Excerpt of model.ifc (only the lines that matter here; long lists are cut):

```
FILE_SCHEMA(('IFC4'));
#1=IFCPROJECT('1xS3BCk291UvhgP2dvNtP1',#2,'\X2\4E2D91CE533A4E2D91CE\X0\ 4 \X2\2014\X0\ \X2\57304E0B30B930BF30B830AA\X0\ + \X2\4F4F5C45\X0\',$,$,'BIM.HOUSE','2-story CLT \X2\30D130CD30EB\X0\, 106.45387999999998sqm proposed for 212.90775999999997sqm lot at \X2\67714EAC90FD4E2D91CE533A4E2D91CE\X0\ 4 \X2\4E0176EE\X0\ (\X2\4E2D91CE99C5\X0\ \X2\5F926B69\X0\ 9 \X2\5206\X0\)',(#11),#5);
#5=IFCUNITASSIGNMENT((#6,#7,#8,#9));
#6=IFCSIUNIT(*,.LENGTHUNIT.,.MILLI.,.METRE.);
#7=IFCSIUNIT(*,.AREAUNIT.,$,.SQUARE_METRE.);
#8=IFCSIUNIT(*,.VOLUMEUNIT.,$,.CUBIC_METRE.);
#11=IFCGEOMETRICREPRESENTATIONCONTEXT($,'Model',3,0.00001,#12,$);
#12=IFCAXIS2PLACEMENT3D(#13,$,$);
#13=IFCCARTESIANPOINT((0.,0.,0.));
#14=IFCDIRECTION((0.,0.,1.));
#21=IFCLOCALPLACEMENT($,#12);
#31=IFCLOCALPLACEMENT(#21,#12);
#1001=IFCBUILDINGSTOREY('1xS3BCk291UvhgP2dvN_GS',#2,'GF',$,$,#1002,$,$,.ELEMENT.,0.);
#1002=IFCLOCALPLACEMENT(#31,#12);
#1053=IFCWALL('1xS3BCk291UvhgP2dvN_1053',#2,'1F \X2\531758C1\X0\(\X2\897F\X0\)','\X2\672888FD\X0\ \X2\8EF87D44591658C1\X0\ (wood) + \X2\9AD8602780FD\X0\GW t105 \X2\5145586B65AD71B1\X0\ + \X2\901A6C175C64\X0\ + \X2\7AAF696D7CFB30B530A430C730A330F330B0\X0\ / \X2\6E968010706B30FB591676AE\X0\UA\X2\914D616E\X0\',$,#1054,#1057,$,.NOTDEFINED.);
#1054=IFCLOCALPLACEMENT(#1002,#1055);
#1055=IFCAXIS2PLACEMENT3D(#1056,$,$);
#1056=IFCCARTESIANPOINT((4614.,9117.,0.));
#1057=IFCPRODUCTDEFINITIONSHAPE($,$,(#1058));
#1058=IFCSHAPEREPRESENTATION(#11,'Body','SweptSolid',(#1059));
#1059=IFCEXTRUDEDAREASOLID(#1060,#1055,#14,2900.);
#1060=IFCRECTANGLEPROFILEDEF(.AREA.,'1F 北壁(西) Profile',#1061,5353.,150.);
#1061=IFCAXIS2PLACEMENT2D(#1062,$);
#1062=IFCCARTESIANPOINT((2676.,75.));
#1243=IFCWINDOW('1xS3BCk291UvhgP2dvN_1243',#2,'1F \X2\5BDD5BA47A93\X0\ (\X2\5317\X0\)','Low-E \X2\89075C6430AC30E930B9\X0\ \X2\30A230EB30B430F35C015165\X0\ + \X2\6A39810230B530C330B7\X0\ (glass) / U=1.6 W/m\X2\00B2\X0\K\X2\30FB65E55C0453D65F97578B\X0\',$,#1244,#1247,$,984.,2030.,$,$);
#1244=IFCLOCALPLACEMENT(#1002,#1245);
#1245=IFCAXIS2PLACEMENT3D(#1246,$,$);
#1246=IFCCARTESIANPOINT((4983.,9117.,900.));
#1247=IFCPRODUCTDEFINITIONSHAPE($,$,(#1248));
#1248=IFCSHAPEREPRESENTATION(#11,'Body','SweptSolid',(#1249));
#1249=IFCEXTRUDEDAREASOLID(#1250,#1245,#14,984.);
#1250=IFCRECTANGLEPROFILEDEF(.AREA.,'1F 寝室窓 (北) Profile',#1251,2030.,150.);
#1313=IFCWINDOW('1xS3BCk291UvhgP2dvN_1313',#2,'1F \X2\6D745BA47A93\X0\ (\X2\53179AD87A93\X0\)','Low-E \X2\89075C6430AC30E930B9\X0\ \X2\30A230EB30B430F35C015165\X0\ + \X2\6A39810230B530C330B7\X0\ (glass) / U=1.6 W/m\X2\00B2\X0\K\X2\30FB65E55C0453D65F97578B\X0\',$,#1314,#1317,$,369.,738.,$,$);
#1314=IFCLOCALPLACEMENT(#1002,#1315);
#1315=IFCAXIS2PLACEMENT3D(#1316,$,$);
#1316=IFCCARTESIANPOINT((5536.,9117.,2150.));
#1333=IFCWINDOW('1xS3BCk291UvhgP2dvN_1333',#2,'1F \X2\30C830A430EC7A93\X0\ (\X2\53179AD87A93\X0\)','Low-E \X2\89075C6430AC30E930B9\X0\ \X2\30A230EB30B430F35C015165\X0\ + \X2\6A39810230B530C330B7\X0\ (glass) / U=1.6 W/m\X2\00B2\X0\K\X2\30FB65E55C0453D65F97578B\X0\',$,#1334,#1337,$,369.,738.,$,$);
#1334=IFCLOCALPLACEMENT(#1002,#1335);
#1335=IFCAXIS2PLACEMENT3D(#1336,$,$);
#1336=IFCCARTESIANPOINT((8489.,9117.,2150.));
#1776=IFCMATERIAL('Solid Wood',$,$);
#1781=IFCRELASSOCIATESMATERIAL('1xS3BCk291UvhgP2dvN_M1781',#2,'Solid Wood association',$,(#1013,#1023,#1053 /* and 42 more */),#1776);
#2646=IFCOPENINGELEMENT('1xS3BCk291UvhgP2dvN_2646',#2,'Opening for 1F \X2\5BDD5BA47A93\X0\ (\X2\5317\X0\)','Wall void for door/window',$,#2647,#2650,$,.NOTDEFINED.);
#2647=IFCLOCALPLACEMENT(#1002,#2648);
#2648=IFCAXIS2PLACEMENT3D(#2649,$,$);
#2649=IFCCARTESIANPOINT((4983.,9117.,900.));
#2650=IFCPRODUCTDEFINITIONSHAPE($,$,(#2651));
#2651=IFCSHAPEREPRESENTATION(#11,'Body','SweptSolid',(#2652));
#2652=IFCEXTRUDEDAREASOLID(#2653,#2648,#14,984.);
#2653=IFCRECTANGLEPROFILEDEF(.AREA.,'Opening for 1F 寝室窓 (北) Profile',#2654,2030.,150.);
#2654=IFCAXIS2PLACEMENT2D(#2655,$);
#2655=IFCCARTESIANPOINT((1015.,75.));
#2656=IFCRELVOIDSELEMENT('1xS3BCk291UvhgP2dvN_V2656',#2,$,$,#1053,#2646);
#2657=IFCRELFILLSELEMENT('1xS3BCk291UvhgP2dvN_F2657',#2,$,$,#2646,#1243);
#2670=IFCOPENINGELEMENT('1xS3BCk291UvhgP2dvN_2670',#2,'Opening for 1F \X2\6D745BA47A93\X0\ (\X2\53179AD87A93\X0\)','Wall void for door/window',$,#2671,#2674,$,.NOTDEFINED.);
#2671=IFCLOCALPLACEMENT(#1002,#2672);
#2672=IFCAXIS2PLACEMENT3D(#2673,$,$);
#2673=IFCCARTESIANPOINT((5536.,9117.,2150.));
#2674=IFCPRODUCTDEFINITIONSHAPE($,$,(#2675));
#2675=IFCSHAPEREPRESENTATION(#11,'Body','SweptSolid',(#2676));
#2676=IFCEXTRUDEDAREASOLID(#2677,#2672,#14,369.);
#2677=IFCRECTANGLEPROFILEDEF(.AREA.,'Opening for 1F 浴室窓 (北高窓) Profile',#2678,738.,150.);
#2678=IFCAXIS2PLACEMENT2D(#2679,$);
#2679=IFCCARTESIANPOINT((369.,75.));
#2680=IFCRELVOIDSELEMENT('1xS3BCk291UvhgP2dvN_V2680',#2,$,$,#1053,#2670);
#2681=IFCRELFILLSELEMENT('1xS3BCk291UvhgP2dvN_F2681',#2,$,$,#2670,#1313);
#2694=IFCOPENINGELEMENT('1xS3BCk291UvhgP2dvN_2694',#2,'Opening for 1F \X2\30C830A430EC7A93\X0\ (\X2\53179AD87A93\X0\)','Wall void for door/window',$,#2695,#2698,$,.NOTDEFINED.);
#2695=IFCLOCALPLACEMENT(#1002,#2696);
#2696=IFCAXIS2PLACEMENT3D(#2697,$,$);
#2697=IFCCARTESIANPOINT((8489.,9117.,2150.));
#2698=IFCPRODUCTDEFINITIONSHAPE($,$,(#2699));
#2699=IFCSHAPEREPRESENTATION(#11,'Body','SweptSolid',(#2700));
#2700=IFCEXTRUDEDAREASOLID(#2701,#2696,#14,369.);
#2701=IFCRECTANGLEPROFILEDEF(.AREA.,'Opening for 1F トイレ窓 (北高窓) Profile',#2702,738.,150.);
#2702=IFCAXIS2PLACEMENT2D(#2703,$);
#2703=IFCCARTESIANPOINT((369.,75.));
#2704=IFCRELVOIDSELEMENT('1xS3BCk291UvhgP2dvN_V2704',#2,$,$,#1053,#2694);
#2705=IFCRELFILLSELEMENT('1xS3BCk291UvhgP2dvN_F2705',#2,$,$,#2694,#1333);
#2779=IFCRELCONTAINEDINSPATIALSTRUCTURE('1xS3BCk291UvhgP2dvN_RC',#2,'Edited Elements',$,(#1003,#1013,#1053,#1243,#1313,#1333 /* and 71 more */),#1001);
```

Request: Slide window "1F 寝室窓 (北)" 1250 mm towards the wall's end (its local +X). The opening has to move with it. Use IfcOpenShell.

```python
import ifcopenshell
import ifcopenshell.api.geometry
import ifcopenshell.util.placement
import ifcopenshell.util.unit

model = ifcopenshell.open("model.ifc")
unit_scale = ifcopenshell.util.unit.calculate_unit_scale(model)

window = model.by_id(1243)
opening = window.FillsVoids[0].RelatingOpeningElement
wall = opening.VoidsElements[0].RelatingBuildingElement

wall_matrix = ifcopenshell.util.placement.get_local_placement(wall.ObjectPlacement)
shift = wall_matrix[:3, 0] * 1.25 / unit_scale
before = ifcopenshell.util.placement.get_local_placement(window.ObjectPlacement)[:3, 3].copy()

# The window is not placed relative to its opening, so move both.
for product in (opening, window):
    matrix = ifcopenshell.util.placement.get_local_placement(product.ObjectPlacement)
    matrix[:3, 3] += shift
    ifcopenshell.api.geometry.edit_object_placement(model, product=product, matrix=matrix, is_si=False)

after = ifcopenshell.util.placement.get_local_placement(window.ObjectPlacement)[:3, 3]
print("window moved by", (after - before).round(3) + 0.0)

model.write("model_updated.ifc")
```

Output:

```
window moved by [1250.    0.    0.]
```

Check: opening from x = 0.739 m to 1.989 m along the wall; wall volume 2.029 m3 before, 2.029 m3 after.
